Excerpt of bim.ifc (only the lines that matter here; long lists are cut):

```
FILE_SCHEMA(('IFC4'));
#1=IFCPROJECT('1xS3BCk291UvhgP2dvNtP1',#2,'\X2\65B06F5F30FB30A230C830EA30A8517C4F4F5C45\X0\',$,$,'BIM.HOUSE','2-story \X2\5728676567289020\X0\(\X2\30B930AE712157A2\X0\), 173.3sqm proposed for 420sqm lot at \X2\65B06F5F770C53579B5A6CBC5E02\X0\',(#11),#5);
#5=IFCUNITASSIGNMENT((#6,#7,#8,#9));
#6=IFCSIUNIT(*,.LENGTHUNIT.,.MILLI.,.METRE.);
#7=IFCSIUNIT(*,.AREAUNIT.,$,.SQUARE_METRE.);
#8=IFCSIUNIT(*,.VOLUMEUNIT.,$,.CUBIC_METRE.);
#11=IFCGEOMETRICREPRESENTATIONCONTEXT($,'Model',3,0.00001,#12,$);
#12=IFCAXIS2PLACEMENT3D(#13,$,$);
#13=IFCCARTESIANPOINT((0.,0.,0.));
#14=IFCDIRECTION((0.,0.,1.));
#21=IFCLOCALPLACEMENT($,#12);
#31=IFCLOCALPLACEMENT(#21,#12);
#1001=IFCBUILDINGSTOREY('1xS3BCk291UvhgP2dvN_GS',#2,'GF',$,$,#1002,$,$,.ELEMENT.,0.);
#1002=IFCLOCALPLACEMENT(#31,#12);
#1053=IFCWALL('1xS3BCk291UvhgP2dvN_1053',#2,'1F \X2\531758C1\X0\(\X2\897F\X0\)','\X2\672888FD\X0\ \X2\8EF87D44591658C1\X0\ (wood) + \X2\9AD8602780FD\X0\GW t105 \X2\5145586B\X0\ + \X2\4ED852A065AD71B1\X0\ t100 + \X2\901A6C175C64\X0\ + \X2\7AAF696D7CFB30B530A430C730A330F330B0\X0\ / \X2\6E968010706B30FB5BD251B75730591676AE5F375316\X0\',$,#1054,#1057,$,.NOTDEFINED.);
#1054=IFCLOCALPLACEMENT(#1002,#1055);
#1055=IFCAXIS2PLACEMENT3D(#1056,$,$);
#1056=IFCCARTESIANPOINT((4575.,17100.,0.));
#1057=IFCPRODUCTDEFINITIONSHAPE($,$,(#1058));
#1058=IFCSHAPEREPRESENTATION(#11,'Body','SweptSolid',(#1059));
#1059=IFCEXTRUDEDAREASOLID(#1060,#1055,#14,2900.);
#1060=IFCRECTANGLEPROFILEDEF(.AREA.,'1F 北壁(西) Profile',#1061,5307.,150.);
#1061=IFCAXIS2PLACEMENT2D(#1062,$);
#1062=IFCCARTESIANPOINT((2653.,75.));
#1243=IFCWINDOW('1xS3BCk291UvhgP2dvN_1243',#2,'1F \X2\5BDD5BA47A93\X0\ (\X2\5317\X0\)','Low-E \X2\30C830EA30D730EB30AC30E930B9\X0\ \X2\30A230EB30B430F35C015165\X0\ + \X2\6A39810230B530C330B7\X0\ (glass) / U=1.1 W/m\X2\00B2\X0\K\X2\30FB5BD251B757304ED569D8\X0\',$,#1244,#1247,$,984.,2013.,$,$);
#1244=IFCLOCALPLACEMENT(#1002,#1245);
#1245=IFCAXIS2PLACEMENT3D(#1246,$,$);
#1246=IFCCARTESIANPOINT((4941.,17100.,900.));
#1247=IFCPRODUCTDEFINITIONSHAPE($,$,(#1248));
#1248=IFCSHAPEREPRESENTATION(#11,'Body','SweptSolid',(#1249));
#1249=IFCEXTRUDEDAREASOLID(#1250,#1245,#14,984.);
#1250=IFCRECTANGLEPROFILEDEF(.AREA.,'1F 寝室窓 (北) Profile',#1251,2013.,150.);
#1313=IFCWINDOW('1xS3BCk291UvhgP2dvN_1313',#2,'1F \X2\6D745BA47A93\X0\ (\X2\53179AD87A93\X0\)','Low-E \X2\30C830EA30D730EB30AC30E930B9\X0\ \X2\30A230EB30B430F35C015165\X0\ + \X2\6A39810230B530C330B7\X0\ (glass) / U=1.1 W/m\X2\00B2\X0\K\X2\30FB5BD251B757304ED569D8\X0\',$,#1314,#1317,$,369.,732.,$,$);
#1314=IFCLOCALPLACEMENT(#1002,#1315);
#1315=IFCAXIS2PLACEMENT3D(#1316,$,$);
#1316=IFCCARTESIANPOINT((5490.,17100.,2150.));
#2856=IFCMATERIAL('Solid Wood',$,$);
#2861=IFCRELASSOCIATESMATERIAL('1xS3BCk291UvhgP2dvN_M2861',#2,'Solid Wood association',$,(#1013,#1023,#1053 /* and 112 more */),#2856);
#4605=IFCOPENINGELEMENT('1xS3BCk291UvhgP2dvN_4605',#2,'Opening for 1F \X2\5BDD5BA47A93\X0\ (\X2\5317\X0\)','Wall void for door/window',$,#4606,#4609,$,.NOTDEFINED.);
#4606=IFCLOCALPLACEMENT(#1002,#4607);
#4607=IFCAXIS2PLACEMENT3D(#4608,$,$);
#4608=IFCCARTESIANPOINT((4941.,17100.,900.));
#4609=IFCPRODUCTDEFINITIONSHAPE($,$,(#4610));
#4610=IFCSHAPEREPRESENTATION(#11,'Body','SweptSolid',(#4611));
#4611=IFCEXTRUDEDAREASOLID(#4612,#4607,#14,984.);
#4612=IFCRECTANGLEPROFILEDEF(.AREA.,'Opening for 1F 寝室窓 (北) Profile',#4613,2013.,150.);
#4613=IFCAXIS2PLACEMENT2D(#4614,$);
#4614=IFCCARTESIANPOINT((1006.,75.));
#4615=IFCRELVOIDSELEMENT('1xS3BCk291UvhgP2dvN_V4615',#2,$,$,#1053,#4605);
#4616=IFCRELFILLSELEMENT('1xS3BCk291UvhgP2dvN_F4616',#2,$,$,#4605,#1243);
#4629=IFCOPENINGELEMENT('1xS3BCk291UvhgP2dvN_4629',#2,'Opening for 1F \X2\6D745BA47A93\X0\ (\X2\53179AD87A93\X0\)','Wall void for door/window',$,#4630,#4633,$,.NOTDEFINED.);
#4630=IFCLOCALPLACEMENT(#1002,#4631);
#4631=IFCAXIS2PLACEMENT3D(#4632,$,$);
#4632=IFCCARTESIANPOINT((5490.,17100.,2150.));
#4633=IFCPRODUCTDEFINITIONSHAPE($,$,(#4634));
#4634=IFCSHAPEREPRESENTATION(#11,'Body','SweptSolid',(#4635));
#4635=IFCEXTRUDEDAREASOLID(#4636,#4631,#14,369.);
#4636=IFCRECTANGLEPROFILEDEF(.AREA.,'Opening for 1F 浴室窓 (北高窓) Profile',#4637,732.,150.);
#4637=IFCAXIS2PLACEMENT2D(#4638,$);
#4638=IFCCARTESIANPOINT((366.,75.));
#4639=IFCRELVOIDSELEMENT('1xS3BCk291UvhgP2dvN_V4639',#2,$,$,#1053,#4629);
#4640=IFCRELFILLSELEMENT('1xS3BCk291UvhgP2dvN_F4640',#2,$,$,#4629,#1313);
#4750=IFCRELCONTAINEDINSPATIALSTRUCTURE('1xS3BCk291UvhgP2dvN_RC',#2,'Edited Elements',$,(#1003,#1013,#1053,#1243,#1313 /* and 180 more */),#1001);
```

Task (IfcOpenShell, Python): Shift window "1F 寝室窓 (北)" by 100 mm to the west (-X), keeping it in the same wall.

```python
import ifcopenshell
import ifcopenshell.api.geometry
import ifcopenshell.util.placement
import ifcopenshell.util.unit

model = ifcopenshell.open("bim.ifc")
unit_scale = ifcopenshell.util.unit.calculate_unit_scale(model)

window = model.by_id(1243)
opening = window.FillsVoids[0].RelatingOpeningElement
wall = opening.VoidsElements[0].RelatingBuildingElement

wall_matrix = ifcopenshell.util.placement.get_local_placement(wall.ObjectPlacement)
shift = wall_matrix[:3, 0] * -0.1 / unit_scale
before = ifcopenshell.util.placement.get_local_placement(window.ObjectPlacement)[:3, 3].copy()

# The window is not placed relative to its opening, so move both.
for product in (opening, window):
    matrix = ifcopenshell.util.placement.get_local_placement(product.ObjectPlacement)
    matrix[:3, 3] += shift
    ifcopenshell.api.geometry.edit_object_placement(model, product=product, matrix=matrix, is_si=False)

after = ifcopenshell.util.placement.get_local_placement(window.ObjectPlacement)[:3, 3]
print("window moved by", (after - before).round(3) + 0.0)

model.write("bim_updated.ifc")
```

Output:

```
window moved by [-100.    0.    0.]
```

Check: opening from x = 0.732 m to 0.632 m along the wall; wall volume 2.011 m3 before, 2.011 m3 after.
